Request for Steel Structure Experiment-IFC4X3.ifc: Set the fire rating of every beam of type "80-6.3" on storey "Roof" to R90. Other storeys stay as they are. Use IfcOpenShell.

First a look at what the model holds.

```python
import ifcopenshell
import ifcopenshell.util.element

model = ifcopenshell.open("Steel Structure Experiment-IFC4X3.ifc")
print(model.schema)
storey = next(s for s in model.by_type("IfcBuildingStorey") if s.Name == "Roof")
beams = [e for e in ifcopenshell.util.element.get_decomposition(storey) if e.is_a("IfcBeam")]
seen = {}
for e in beams:
    element_type = ifcopenshell.util.element.get_type(e)
    key = (element_type.Name if element_type != e and element_type else None, ifcopenshell.util.element.get_pset(e, "Pset_BeamCommon", "FireRating"))
    seen[key] = seen.get(key, 0) + 1
for (name, value), count in sorted(seen.items(), key=str):
    print(count, "x", name, "|", value)
```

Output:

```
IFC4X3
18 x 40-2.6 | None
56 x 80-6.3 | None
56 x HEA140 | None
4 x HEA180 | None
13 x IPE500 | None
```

```python
import ifcopenshell
import ifcopenshell.api.pset
import ifcopenshell.util.element

model = ifcopenshell.open("Steel Structure Experiment-IFC4X3.ifc")

storey = next(s for s in model.by_type("IfcBuildingStorey") if s.Name == "Roof")
beams = [e for e in ifcopenshell.util.element.get_decomposition(storey) if e.is_a("IfcBeam")]

count = 0
for e in beams:
    element_type = ifcopenshell.util.element.get_type(e)
    if element_type in (None, e) or element_type.Name != "80-6.3":
        continue
    # add_pset returns the element's existing set when there is one.
    pset = ifcopenshell.api.pset.add_pset(model, product=e, name="Pset_BeamCommon")
    ifcopenshell.api.pset.edit_pset(model, pset=pset, properties={"FireRating": "R90"})
    count += 1

print(count, "beams updated")

model.write("Steel Structure Experiment-IFC4X3_updated.ifc")
```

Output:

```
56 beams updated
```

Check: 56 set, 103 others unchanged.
